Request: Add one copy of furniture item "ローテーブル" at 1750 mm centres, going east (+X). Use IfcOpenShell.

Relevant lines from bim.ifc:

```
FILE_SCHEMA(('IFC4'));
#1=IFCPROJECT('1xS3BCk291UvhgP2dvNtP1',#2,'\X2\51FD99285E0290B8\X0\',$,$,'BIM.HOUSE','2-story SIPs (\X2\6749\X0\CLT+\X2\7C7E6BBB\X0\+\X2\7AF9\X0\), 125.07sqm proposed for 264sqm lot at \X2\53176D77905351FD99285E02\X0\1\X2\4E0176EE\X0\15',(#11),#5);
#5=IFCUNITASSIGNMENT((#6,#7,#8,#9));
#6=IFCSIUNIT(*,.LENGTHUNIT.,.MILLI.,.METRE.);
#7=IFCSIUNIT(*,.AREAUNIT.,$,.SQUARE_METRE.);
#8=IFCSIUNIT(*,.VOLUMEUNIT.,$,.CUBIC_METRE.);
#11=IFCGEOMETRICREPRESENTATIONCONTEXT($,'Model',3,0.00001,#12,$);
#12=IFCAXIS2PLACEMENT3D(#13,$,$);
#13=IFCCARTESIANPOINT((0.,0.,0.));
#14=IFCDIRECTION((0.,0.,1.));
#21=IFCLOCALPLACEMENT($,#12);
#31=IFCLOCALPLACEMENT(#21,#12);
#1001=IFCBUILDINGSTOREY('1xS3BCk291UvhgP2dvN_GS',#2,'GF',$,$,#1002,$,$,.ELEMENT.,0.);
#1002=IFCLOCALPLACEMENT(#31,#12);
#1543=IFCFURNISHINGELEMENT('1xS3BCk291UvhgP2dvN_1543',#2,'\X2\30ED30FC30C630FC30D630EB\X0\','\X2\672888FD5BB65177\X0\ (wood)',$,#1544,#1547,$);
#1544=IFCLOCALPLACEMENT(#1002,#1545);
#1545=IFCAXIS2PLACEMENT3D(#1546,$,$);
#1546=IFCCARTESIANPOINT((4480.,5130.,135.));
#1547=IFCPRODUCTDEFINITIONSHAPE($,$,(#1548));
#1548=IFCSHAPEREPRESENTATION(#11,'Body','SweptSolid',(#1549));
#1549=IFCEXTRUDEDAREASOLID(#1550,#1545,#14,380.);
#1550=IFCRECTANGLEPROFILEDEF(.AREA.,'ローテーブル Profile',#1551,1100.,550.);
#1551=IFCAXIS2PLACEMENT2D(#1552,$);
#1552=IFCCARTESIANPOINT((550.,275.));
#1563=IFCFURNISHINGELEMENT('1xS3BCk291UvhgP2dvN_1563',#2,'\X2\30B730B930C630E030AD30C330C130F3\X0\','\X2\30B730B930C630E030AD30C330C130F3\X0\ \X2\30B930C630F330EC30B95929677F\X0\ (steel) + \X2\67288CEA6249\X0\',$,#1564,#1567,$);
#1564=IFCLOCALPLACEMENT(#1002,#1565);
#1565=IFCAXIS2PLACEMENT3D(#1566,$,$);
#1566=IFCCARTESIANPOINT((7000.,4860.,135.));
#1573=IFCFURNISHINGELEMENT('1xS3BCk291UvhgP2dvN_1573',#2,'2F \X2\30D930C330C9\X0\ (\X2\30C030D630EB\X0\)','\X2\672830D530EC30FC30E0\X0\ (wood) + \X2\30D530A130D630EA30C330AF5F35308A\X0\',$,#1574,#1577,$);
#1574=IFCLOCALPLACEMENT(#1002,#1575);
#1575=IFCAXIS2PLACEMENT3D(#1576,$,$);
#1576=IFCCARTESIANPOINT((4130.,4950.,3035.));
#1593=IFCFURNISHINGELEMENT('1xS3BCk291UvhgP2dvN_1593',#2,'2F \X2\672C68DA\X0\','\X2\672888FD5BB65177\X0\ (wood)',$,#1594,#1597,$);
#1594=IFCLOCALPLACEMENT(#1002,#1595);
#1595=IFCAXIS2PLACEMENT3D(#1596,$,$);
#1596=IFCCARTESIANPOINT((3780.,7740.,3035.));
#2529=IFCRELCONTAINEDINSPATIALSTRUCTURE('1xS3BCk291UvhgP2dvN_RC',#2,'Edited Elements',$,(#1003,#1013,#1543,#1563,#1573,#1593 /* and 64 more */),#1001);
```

```python
import numpy as np
import ifcopenshell
import ifcopenshell.api.geometry
import ifcopenshell.api.root
import ifcopenshell.util.element
import ifcopenshell.util.placement
import ifcopenshell.util.unit

model = ifcopenshell.open("bim.ifc")
unit_scale = ifcopenshell.util.unit.calculate_unit_scale(model)


def reuse_history(source, copy):
    """copy_class also copies each property set's owner history, people and application; keep the originals."""
    for rel in copy.IsDefinedBy:
        if rel.is_a("IfcRelDefinesByProperties") and (history := rel.RelatingPropertyDefinition.OwnerHistory):
            rel.RelatingPropertyDefinition.OwnerHistory = source.OwnerHistory
            ifcopenshell.util.element.remove_deep2(model, history)


source = model.by_guid("1xS3BCk291UvhgP2dvN_1543")
base = ifcopenshell.util.placement.get_local_placement(source.ObjectPlacement)
step = np.array([1.0, 0.0, 0.0]) * 1.75 / unit_scale

for i in range(1, 2):
    copy = ifcopenshell.api.root.copy_class(model, product=source)
    copy.Representation = ifcopenshell.util.element.copy_deep(
        model, source.Representation, exclude=["IfcGeometricRepresentationContext", "IfcRepresentationMap"]
    )
    reuse_history(source, copy)
    matrix = base.copy()
    matrix[:3, 3] += i * step
    print("added at", matrix[:3, 3].round(3) + 0.0)
    ifcopenshell.api.geometry.edit_object_placement(model, product=copy, matrix=matrix, is_si=False)

model.write("bim-out.ifc")
```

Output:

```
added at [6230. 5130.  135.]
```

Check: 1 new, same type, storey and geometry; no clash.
